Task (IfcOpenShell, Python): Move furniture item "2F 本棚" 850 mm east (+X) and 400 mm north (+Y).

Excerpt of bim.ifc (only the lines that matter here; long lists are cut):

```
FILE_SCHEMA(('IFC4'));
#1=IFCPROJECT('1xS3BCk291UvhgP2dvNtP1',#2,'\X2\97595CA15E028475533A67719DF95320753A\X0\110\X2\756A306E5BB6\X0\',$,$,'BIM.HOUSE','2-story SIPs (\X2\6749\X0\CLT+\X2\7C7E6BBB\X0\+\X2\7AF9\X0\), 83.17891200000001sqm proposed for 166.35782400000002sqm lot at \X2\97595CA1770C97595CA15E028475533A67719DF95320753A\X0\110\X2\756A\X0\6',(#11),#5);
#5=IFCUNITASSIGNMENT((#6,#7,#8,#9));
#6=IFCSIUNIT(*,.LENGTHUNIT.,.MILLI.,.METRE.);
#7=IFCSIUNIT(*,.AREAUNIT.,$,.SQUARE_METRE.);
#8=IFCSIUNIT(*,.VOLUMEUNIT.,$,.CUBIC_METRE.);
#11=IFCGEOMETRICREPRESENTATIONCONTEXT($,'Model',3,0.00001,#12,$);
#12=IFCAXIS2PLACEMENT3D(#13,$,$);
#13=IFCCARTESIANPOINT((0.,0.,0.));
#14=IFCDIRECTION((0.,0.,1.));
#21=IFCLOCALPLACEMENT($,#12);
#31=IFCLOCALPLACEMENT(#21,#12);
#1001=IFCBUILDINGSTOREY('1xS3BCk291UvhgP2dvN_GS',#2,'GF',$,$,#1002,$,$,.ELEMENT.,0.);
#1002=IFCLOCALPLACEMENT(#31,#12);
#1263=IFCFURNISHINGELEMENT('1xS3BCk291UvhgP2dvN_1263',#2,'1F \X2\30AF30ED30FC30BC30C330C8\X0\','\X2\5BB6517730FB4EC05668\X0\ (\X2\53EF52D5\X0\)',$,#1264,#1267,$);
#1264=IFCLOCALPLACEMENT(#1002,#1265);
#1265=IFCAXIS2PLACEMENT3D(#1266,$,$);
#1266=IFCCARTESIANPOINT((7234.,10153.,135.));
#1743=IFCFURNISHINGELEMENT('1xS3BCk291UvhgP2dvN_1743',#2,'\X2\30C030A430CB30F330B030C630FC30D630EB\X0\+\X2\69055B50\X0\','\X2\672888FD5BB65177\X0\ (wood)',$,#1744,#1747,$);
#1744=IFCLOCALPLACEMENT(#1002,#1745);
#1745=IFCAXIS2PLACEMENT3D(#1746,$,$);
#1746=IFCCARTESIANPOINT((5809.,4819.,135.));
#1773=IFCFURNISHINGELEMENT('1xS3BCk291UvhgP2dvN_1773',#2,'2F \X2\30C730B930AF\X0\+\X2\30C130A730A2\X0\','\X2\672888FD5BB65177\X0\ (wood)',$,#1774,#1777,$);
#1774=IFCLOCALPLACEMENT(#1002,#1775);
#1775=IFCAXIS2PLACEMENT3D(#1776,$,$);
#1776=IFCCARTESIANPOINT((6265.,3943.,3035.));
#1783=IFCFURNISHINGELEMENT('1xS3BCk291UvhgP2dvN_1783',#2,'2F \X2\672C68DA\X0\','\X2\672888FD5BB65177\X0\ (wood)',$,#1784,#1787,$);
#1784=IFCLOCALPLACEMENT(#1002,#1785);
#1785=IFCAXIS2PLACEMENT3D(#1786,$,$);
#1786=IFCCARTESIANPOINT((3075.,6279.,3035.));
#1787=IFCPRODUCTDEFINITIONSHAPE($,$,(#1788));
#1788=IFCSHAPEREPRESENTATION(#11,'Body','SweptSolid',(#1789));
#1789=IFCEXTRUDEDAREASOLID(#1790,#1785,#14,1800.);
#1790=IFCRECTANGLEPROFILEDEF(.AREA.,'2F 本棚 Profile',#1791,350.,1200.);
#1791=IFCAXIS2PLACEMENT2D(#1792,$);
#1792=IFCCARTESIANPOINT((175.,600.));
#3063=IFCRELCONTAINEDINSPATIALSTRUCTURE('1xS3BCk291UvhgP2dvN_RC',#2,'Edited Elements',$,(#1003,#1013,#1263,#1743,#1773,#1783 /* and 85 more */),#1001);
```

```python
import ifcopenshell
import ifcopenshell.api.geometry
import ifcopenshell.util.placement
import ifcopenshell.util.unit

model = ifcopenshell.open("bim.ifc")
unit_scale = ifcopenshell.util.unit.calculate_unit_scale(model)

item = model.by_id(1783)
matrix = ifcopenshell.util.placement.get_local_placement(item.ObjectPlacement)
matrix[0, 3] += 0.85 / unit_scale
matrix[1, 3] += 0.4 / unit_scale
ifcopenshell.api.geometry.edit_object_placement(model, product=item, matrix=matrix, is_si=False)

print(ifcopenshell.util.placement.get_local_placement(item.ObjectPlacement).round(3) + 0.0)

model.write("bim_rev.ifc")
```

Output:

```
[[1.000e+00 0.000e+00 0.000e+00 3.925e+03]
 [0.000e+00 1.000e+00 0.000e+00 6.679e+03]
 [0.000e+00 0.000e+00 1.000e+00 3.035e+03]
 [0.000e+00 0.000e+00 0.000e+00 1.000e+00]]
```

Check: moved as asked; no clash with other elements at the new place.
